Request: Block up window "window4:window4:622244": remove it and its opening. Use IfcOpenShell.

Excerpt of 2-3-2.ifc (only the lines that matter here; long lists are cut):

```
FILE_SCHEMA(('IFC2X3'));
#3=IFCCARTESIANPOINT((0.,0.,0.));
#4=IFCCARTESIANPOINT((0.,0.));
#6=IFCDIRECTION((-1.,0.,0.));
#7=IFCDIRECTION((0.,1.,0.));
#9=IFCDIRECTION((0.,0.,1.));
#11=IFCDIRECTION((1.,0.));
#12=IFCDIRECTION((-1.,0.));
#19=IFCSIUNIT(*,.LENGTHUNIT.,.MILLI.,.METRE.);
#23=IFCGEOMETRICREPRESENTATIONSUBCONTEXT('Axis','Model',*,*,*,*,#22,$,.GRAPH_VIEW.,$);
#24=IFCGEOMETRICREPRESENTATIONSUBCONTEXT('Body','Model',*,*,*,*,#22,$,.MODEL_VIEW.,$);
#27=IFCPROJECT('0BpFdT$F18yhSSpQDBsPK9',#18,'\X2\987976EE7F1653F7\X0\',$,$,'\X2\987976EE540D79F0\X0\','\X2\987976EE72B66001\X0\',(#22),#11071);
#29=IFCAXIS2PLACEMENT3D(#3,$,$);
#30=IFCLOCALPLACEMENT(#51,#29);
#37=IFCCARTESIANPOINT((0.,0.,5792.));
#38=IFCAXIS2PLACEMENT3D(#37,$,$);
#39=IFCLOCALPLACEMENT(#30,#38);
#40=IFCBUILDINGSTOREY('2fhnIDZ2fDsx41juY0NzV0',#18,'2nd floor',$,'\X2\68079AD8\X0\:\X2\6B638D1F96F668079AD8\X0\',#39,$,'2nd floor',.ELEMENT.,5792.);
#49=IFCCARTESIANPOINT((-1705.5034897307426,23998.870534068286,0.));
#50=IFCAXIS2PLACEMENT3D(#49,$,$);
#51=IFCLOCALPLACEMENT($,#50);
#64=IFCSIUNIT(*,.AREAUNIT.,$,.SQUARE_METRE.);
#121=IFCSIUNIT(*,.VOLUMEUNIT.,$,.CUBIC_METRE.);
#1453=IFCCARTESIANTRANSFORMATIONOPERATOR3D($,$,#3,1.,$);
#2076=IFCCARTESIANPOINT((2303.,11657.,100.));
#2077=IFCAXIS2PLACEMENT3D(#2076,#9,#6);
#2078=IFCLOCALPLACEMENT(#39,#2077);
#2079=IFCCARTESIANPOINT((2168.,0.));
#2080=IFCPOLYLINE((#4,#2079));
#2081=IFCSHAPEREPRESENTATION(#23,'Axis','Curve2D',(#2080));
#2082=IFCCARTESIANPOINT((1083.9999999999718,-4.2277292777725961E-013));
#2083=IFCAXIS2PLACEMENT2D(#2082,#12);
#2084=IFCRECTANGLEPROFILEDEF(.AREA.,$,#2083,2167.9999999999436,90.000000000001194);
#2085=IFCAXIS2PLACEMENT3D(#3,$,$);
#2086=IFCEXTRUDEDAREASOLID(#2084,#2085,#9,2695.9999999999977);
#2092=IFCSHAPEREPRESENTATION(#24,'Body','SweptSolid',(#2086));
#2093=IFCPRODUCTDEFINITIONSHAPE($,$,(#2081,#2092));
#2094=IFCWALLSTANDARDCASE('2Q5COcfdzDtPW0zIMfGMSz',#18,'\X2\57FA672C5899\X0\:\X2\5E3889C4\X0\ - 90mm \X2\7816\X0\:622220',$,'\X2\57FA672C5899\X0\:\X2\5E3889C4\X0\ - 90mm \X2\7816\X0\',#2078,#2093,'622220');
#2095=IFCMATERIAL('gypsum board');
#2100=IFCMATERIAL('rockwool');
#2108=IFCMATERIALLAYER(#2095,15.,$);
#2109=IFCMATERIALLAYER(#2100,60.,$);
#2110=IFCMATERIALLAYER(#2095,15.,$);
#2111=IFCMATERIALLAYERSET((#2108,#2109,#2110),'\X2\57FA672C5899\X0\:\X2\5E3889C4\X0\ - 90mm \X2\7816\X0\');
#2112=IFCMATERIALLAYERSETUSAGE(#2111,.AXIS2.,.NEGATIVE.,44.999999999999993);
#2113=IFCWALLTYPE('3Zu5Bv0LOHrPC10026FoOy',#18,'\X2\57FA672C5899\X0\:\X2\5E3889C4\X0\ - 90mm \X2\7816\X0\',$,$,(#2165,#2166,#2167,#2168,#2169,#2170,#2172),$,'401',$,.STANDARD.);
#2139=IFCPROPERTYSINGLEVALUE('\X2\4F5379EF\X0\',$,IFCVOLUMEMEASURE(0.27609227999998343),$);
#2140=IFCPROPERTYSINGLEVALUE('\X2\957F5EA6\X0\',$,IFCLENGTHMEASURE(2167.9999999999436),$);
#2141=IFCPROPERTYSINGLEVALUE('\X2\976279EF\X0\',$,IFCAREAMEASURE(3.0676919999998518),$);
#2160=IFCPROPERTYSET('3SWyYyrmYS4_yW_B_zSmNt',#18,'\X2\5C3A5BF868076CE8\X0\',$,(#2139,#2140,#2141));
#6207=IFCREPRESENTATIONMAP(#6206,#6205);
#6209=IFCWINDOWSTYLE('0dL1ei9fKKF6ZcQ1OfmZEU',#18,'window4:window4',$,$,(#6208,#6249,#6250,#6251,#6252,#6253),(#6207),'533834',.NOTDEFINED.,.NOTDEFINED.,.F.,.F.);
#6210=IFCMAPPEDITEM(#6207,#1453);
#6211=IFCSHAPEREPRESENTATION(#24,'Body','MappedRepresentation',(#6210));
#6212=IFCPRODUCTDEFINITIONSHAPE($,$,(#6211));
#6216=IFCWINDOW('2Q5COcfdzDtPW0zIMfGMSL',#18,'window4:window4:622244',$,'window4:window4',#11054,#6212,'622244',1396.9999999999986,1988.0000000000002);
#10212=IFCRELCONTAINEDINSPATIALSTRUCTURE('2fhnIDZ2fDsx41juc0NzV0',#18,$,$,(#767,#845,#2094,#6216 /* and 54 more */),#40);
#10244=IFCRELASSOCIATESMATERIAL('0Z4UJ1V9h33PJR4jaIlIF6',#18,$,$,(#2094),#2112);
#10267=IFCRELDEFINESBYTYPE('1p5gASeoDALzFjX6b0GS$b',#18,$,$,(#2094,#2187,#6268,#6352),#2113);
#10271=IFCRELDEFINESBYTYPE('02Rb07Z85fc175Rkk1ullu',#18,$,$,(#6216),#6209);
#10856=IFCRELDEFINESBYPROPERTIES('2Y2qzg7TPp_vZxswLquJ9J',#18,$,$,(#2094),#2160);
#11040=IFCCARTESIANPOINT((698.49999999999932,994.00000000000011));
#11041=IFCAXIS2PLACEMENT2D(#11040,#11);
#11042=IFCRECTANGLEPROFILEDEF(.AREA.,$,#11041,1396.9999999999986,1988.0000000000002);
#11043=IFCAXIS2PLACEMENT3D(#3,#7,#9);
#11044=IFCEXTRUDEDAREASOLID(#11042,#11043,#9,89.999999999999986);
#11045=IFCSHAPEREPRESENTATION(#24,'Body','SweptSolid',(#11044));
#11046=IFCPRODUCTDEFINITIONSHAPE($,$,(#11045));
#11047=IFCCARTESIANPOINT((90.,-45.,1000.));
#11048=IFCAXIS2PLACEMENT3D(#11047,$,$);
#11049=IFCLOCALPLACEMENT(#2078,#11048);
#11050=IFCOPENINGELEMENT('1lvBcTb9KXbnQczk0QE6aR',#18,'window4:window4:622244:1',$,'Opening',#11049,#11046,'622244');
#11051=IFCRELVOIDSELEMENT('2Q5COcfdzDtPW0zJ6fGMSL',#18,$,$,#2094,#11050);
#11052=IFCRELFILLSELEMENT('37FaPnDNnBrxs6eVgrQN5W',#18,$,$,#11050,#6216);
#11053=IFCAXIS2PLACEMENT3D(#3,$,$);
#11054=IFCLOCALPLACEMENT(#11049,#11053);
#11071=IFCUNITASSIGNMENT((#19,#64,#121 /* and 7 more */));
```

```python
import ifcopenshell
import ifcopenshell.api.feature
import ifcopenshell.api.pset
import ifcopenshell.api.root
import ifcopenshell.geom
import ifcopenshell.util.element
import ifcopenshell.util.shape
import ifcopenshell.util.unit

model = ifcopenshell.open("2-3-2.ifc")
area_scale = ifcopenshell.util.unit.calculate_unit_scale(model, "AREAUNIT")
volume_scale = ifcopenshell.util.unit.calculate_unit_scale(model, "VOLUMEUNIT")
settings = ifcopenshell.geom.settings()


def volume(element):
    """Net volume in cubic metres, openings subtracted."""
    shape = ifcopenshell.geom.create_shape(settings, element)
    return ifcopenshell.util.shape.get_volume(shape.geometry)


window = model.by_guid("2Q5COcfdzDtPW0zIMfGMSL")
opening = window.FillsVoids[0].RelatingOpeningElement
wall = opening.VoidsElements[0].RelatingBuildingElement
before = volume(wall)

ifcopenshell.api.root.remove_product(model, product=window)
ifcopenshell.api.feature.remove_feature(model, feature=opening)

after = volume(wall)
thickness = 0.09  # wall thickness in metres

# Update the wall's stored quantities.
pset = model.by_id(ifcopenshell.util.element.get_pset(wall, "尺寸标注", should_inherit=False)["id"])
ifcopenshell.api.pset.edit_pset(model, pset=pset, properties={
    "体积": model.create_entity("IfcVolumeMeasure", after / volume_scale),
    "面积": model.create_entity("IfcAreaMeasure", after / thickness / area_scale),
})

print(f"wall volume {before:.3f} -> {after:.3f} m3")

model.write("2-3-2-out.ifc")
```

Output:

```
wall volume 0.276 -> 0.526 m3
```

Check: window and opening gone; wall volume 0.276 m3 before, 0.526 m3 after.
